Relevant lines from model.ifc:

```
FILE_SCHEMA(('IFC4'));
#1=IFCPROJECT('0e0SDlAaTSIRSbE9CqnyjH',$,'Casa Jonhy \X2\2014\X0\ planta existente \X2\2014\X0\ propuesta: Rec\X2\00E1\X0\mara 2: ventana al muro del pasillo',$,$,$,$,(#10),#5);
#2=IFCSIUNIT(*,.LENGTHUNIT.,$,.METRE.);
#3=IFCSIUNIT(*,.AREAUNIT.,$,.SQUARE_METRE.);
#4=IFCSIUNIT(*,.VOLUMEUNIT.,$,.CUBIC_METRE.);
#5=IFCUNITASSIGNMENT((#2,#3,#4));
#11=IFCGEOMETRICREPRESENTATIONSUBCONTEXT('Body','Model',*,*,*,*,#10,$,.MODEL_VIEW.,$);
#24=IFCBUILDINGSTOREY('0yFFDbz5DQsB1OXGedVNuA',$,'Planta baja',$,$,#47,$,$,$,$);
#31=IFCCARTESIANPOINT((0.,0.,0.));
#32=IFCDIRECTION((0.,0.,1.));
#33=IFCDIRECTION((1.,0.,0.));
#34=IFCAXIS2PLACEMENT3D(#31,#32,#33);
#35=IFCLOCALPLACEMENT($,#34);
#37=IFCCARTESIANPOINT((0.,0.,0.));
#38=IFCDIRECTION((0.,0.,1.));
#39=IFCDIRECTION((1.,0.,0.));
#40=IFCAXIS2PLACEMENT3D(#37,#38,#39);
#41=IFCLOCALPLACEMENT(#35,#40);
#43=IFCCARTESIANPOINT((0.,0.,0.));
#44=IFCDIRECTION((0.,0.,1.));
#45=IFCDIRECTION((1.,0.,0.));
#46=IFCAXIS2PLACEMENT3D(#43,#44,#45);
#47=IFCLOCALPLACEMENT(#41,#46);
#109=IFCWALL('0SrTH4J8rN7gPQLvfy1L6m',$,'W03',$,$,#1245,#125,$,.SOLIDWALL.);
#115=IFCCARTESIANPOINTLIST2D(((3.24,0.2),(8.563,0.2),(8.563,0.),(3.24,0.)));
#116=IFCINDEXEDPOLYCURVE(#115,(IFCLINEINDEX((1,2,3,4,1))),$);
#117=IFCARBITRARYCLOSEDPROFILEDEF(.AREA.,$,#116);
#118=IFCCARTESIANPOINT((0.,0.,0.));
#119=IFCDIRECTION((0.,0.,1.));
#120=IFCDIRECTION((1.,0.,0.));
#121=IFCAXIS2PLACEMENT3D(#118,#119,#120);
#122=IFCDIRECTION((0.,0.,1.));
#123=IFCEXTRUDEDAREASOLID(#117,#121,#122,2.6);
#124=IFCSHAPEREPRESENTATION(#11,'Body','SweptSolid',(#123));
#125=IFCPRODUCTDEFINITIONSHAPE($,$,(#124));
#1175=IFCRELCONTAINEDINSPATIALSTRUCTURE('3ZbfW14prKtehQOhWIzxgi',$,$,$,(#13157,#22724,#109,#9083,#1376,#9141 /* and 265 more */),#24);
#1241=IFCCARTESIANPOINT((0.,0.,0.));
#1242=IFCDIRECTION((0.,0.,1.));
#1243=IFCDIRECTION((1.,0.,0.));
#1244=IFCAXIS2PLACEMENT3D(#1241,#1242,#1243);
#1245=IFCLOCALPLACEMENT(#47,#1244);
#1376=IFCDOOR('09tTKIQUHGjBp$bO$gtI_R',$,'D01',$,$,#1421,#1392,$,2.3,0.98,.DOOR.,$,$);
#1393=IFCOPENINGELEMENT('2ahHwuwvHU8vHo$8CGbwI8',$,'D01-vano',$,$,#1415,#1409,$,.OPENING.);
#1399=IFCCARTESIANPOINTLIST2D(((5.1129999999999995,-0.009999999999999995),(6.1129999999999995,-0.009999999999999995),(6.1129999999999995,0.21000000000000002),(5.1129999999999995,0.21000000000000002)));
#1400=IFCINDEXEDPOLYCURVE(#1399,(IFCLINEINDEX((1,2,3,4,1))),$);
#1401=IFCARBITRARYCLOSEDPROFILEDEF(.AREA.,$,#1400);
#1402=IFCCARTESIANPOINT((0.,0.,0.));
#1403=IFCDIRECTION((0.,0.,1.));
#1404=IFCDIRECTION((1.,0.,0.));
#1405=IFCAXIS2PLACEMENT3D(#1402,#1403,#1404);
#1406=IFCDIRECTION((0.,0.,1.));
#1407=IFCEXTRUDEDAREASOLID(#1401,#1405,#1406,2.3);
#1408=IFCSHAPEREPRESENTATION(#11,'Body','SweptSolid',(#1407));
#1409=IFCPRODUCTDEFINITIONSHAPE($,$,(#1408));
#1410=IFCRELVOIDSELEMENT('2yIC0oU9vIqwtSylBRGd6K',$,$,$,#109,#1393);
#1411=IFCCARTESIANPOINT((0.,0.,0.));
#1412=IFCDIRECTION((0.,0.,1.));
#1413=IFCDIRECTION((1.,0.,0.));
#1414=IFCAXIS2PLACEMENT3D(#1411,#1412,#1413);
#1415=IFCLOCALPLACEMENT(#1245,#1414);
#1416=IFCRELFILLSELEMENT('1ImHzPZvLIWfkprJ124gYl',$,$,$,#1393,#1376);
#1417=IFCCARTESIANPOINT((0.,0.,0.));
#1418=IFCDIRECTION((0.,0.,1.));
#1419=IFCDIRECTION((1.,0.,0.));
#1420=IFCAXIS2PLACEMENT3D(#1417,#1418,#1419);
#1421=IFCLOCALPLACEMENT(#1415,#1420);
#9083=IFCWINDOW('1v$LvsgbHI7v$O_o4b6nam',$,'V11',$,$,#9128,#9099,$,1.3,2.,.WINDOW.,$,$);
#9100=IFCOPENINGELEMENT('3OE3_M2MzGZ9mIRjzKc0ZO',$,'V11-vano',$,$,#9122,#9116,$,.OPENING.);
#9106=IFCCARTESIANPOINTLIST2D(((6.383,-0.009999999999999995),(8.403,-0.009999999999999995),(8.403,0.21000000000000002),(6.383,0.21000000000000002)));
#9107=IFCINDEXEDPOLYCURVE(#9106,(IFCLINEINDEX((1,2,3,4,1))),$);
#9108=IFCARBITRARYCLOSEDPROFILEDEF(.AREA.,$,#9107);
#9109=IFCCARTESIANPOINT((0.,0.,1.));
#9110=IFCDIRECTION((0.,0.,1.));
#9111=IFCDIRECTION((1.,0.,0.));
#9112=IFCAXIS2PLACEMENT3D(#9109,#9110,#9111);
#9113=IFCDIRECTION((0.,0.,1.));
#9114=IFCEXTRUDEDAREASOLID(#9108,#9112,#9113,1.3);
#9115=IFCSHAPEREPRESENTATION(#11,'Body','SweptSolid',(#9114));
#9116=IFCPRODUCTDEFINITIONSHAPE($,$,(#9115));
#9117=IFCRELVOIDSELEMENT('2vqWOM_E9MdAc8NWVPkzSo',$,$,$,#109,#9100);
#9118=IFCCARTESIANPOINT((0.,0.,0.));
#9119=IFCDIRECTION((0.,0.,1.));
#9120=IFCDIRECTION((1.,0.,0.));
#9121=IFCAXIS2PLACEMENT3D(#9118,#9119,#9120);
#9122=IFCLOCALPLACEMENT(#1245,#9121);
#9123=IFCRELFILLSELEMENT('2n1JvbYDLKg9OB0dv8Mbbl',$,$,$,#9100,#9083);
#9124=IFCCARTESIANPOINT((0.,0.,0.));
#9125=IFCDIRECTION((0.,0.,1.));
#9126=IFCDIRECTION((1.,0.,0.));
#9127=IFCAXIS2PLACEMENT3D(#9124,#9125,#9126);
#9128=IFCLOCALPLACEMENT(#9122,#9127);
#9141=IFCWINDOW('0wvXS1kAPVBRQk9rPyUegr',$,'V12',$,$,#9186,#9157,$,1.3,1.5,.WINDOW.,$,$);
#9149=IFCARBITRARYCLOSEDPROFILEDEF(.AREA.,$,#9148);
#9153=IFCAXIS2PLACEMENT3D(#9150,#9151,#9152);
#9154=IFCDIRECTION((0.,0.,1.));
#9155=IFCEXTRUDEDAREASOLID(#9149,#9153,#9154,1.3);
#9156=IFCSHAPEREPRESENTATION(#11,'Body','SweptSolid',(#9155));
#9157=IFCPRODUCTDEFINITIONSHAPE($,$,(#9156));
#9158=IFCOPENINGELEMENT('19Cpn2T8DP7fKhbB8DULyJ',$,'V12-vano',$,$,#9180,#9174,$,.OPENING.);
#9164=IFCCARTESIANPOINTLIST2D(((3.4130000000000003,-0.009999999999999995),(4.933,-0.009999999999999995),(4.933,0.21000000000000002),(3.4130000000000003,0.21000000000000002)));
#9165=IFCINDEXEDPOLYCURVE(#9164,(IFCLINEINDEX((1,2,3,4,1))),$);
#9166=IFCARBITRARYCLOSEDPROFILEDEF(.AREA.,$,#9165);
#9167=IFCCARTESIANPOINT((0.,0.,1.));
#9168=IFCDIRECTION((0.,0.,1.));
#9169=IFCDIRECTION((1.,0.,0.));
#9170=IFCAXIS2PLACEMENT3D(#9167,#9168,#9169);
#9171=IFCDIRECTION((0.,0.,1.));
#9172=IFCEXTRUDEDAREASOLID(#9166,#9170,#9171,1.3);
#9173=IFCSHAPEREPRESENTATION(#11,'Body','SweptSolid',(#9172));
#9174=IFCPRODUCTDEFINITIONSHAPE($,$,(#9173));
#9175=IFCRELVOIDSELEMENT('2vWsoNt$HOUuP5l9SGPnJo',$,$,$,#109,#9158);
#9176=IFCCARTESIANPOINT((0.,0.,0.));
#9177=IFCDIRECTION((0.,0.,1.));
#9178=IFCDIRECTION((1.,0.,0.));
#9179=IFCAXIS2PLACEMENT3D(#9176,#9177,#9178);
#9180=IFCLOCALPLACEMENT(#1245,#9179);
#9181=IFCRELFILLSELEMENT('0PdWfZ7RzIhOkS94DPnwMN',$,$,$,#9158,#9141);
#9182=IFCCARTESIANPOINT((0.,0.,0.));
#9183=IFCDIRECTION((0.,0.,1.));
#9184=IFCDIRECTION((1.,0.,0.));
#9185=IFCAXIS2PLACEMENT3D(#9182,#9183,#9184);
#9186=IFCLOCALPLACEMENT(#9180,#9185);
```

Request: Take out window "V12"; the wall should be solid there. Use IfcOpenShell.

```python
import ifcopenshell
import ifcopenshell.api.feature
import ifcopenshell.api.root
import ifcopenshell.geom
import ifcopenshell.util.shape

model = ifcopenshell.open("model.ifc")
settings = ifcopenshell.geom.settings()


def volume(element):
    """Net volume in cubic metres, openings subtracted."""
    shape = ifcopenshell.geom.create_shape(settings, element)
    return ifcopenshell.util.shape.get_volume(shape.geometry)


window = model.by_id(9141)
opening = window.FillsVoids[0].RelatingOpeningElement
wall = opening.VoidsElements[0].RelatingBuildingElement
before = volume(wall)

ifcopenshell.api.root.remove_product(model, product=window)
ifcopenshell.api.feature.remove_feature(model, feature=opening)

after = volume(wall)

print(f"wall volume {before:.3f} -> {after:.3f} m3")

model.write("model_updated.ifc")
```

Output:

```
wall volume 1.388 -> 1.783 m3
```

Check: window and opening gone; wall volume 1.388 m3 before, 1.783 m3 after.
